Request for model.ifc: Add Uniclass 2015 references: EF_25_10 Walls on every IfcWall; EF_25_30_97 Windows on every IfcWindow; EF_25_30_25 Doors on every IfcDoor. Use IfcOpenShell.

First a look at what the model holds.

```python
import ifcopenshell

model = ifcopenshell.open("model.ifc")
print(model.schema)
print("classifications:", [c.Name for c in model.by_type("IfcClassification")])
for ifc_class in ("IfcDoor", "IfcRoof", "IfcStair", "IfcWall", "IfcWindow"):
    print(ifc_class, len(model.by_type(ifc_class)))
```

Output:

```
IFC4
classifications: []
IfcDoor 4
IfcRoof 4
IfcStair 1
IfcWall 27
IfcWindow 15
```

```python
import ifcopenshell
import ifcopenshell.api.classification

model = ifcopenshell.open("model.ifc")

system = ifcopenshell.api.classification.add_classification(model, classification="Uniclass 2015")

codes = {
    "IfcWall": ("EF_25_10", "Walls"),
    "IfcWindow": ("EF_25_30_97", "Windows"),
    "IfcDoor": ("EF_25_30_25", "Doors"),
}
for ifc_class, (code, name) in codes.items():
    products = model.by_type(ifc_class)
    ifcopenshell.api.classification.add_reference(
        model, products=products, classification=system, identification=code, name=name
    )
    print(code, len(products))

model.write("model_rev.ifc")
```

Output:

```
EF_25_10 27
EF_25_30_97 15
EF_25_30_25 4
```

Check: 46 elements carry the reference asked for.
